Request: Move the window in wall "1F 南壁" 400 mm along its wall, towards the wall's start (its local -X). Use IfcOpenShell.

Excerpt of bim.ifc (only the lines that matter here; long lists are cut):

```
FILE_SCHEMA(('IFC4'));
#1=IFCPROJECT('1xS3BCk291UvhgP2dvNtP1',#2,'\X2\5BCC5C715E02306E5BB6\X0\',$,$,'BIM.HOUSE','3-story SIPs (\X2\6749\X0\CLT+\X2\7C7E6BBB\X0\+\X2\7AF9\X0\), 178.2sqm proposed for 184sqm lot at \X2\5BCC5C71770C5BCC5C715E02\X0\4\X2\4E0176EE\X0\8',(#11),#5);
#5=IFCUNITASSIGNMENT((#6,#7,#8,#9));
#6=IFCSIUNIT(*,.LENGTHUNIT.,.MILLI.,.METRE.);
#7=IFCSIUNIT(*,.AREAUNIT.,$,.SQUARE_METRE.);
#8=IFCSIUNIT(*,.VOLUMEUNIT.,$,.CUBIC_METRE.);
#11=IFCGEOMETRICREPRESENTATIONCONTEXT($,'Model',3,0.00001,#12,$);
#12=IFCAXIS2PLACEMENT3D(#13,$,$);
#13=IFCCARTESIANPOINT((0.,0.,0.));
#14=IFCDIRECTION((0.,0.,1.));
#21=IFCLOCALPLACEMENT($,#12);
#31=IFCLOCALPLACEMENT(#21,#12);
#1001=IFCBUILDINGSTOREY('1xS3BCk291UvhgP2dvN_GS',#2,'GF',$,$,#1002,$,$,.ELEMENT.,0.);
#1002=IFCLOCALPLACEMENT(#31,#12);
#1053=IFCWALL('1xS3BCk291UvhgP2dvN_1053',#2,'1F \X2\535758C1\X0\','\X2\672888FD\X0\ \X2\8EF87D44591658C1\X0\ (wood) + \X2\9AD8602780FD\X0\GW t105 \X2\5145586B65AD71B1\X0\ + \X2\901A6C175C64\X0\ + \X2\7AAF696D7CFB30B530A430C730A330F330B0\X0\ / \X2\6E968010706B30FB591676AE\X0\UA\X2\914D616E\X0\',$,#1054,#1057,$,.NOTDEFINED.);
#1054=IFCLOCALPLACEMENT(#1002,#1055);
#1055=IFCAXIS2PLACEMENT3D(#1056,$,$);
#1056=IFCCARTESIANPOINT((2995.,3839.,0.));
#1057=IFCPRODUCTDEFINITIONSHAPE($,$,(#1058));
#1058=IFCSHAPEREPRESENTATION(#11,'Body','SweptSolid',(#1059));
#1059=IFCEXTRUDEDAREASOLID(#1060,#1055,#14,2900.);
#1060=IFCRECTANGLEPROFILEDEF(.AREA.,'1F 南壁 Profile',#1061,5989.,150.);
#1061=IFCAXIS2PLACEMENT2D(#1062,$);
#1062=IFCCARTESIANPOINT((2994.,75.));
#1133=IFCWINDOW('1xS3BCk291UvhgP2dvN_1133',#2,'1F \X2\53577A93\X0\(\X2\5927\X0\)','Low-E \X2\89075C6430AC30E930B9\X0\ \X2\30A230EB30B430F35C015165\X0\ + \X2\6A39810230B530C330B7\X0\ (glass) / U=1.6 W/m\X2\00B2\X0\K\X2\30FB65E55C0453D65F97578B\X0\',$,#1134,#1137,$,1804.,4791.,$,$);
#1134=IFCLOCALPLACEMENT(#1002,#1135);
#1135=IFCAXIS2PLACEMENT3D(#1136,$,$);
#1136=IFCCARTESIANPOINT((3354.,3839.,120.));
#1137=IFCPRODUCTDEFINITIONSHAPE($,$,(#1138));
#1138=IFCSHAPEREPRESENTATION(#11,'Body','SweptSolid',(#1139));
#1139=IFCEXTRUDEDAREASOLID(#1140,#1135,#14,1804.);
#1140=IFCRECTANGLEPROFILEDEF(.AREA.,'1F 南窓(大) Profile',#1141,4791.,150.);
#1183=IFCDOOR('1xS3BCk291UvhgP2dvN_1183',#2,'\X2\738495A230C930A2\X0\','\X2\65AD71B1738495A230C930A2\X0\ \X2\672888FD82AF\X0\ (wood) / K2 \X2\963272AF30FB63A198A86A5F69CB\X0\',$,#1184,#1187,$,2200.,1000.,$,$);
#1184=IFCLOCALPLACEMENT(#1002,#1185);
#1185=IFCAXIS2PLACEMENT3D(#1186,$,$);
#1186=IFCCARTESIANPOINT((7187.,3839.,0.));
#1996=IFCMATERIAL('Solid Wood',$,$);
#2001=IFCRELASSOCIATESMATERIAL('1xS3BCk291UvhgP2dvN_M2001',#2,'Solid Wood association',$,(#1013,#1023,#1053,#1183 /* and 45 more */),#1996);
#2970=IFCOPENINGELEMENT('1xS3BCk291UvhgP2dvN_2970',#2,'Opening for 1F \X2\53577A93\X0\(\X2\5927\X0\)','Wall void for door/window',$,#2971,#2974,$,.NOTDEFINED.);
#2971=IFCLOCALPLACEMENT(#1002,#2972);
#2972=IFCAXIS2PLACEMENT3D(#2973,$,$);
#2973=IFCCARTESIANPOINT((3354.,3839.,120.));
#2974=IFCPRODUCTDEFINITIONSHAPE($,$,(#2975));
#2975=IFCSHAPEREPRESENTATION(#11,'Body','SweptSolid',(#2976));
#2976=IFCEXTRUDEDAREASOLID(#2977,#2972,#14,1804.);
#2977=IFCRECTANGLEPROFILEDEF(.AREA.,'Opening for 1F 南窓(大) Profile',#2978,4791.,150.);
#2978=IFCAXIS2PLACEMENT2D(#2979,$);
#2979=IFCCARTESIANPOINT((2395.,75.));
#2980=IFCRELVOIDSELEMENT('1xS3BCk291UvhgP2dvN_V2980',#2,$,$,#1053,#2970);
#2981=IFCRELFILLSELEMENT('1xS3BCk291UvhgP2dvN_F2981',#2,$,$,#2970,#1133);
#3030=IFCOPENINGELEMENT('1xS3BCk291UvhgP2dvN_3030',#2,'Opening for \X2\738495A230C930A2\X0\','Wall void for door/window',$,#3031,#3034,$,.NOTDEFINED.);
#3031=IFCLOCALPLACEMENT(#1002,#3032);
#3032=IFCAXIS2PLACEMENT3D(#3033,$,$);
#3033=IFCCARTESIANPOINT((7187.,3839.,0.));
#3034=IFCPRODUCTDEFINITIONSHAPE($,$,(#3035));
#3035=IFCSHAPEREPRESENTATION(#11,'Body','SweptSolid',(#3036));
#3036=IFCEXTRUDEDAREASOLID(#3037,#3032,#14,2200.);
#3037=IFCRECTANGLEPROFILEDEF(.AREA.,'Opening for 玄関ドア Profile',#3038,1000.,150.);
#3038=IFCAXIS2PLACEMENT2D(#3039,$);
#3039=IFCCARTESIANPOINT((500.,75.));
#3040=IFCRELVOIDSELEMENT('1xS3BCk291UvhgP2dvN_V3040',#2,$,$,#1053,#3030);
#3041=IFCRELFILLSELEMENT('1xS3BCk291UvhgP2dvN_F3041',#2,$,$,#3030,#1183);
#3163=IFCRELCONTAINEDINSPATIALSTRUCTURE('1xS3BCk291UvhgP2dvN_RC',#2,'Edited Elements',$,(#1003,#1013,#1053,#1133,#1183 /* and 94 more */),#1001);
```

```python
import ifcopenshell
import ifcopenshell.api.geometry
import ifcopenshell.util.placement

model = ifcopenshell.open("bim.ifc")

window = model.by_guid("1xS3BCk291UvhgP2dvN_1133")
opening = window.FillsVoids[0].RelatingOpeningElement
wall = opening.VoidsElements[0].RelatingBuildingElement

wall_matrix = ifcopenshell.util.placement.get_local_placement(wall.ObjectPlacement)
shift = wall_matrix[:3, 0] * -400.0
before = ifcopenshell.util.placement.get_local_placement(window.ObjectPlacement)[:3, 3].copy()

# The window is not placed relative to its opening, so move both.
for product in (opening, window):
    matrix = ifcopenshell.util.placement.get_local_placement(product.ObjectPlacement)
    matrix[:3, 3] += shift
    ifcopenshell.api.geometry.edit_object_placement(model, product=product, matrix=matrix, is_si=False)

after = ifcopenshell.util.placement.get_local_placement(window.ObjectPlacement)[:3, 3]
print("window moved by", (after - before).round(3) + 0.0)

model.write("bim_edited.ifc")
```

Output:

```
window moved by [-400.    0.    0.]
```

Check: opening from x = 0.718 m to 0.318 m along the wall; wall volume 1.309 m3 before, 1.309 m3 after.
